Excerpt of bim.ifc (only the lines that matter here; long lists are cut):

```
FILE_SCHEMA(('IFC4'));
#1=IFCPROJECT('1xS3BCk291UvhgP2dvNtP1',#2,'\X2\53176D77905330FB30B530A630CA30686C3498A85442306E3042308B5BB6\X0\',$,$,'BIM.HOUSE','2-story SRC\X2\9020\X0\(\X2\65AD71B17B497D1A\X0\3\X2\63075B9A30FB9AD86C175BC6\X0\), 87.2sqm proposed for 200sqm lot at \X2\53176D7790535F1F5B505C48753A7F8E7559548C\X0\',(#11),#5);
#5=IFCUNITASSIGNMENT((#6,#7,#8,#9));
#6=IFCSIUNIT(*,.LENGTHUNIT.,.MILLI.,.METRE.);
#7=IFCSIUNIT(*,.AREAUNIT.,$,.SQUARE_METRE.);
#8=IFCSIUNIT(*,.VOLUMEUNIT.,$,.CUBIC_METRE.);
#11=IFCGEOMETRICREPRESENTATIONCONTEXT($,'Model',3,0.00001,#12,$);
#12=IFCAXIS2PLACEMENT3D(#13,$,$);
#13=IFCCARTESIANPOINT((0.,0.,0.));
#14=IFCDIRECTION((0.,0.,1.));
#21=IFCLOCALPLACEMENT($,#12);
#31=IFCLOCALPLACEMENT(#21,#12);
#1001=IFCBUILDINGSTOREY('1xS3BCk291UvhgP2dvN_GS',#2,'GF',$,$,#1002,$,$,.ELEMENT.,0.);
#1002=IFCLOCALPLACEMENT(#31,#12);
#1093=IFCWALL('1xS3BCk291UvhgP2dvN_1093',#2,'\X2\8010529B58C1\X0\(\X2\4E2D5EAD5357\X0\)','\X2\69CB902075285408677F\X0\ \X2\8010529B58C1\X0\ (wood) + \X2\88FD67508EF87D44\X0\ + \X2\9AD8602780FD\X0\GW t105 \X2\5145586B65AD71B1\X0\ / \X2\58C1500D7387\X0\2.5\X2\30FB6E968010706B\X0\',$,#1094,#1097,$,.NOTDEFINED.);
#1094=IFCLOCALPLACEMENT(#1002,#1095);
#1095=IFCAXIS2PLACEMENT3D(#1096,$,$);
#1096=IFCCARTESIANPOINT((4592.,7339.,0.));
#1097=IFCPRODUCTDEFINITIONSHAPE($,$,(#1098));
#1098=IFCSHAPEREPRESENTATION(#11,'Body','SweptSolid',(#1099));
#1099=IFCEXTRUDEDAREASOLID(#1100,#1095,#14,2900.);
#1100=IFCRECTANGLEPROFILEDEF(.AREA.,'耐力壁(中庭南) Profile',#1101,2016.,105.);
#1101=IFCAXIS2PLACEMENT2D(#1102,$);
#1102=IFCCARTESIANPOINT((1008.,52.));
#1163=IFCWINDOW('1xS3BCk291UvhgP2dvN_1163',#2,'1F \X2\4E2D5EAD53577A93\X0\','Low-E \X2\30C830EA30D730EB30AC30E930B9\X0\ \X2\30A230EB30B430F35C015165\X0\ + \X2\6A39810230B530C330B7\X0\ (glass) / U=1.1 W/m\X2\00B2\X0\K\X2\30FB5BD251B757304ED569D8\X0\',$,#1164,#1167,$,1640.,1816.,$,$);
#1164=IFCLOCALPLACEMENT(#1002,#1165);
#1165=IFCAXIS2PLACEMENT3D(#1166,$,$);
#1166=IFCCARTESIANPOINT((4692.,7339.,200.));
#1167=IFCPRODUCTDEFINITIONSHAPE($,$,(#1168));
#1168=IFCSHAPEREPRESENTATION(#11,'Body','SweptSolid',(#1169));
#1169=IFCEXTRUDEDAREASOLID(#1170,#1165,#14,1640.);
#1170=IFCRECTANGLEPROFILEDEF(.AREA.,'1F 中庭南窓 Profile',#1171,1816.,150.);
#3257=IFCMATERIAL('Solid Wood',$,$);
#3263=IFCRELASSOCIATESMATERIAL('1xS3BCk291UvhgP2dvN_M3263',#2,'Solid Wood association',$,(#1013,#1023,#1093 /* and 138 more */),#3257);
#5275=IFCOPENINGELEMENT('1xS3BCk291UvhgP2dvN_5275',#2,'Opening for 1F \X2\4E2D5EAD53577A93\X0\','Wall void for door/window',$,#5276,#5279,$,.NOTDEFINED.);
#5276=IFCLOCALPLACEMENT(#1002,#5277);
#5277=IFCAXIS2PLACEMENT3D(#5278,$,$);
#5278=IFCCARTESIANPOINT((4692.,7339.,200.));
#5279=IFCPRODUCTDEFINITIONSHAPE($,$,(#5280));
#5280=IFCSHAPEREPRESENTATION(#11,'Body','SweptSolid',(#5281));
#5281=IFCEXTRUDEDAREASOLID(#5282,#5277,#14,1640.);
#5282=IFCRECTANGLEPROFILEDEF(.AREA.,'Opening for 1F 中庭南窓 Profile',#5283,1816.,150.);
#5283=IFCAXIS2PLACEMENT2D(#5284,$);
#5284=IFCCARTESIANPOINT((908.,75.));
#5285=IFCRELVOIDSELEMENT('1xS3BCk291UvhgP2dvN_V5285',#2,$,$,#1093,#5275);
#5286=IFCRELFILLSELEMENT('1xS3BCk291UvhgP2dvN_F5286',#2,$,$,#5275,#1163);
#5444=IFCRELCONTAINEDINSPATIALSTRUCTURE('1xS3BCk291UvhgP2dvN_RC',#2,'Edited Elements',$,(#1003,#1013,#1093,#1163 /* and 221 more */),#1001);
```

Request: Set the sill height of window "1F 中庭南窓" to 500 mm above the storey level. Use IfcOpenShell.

```python
import numpy as np
import ifcopenshell
import ifcopenshell.api.geometry
import ifcopenshell.geom
import ifcopenshell.util.element
import ifcopenshell.util.placement
import ifcopenshell.util.shape
import ifcopenshell.util.unit

model = ifcopenshell.open("bim.ifc")
unit_scale = ifcopenshell.util.unit.calculate_unit_scale(model)

window = model.by_id(1163)
opening = window.FillsVoids[0].RelatingOpeningElement
storey = ifcopenshell.util.element.get_container(window, ifc_class="IfcBuildingStorey")
level = ifcopenshell.util.placement.get_local_placement(storey.ObjectPlacement)[2, 3]

# The opening's origin need not be at the sill, so measure its lowest point.
shape = ifcopenshell.geom.create_shape(ifcopenshell.geom.settings(), opening)
bottom = ifcopenshell.util.shape.get_shape_bottom_elevation(shape, shape.geometry) / unit_scale
dz = level + 0.5 / unit_scale - bottom

shift = np.array([0.0, 0.0, dz])
# The window is not placed relative to its opening, so move both.
for product in (opening, window):
    matrix = ifcopenshell.util.placement.get_local_placement(product.ObjectPlacement)
    matrix[:3, 3] += shift
    ifcopenshell.api.geometry.edit_object_placement(model, product=product, matrix=matrix, is_si=False)

print(f"moved by {dz * unit_scale:+.3f} m")

model.write("bim_updated.ifc")
```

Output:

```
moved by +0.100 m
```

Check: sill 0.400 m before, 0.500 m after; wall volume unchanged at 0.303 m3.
